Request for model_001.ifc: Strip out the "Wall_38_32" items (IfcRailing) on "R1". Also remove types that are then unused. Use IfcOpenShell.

First a look at what the model holds.

```python
import ifcopenshell
import ifcopenshell.util.element

model = ifcopenshell.open("model_001.ifc")
print(model.schema)
storey = next(s for s in model.by_type("IfcBuildingStorey") if s.Name == "R1")
railings = [e for e in ifcopenshell.util.element.get_decomposition(storey) if e.is_a("IfcRailing")]
seen = {}
for e in railings:
    element_type = ifcopenshell.util.element.get_type(e)
    name = element_type.Name if element_type not in (None, e) else None
    seen[name] = seen.get(name, 0) + 1
for name, count in sorted(seen.items(), key=str):
    print(count, "x", name)
```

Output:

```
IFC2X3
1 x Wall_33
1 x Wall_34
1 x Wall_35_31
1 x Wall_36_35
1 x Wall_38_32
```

```python
import ifcopenshell
import ifcopenshell.api.root
import ifcopenshell.util.element

model = ifcopenshell.open("model_001.ifc")

storey = next(s for s in model.by_type("IfcBuildingStorey") if s.Name == "R1")
railings = [e for e in ifcopenshell.util.element.get_decomposition(storey) if e.is_a("IfcRailing")]
targets = [e for e in railings if (t := ifcopenshell.util.element.get_type(e)) not in (None, e) and t.Name == "Wall_38_32"]
types = {ifcopenshell.util.element.get_type(e) for e in targets} - {None, *targets}

for e in targets:
    ifcopenshell.api.root.remove_product(model, product=e)
print(len(targets), "removed")

unused = [t for t in types if not ifcopenshell.util.element.get_types(t)]
for t in unused:
    ifcopenshell.api.root.remove_product(model, product=t)
print(len(unused), "unused types removed")

model.write("model_001-out.ifc")
```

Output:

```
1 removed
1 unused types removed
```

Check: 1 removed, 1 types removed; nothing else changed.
